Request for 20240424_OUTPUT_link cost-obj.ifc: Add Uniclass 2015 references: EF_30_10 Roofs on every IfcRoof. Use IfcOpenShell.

First a look at what the model holds.

```python
import ifcopenshell

model = ifcopenshell.open("20240424_OUTPUT_link cost-obj.ifc")
print(model.schema)
print("classifications:", [c.Name for c in model.by_type("IfcClassification")])
for ifc_class in ("IfcDoor", "IfcRoof", "IfcStair", "IfcWall", "IfcWindow"):
    print(ifc_class, len(model.by_type(ifc_class)))
```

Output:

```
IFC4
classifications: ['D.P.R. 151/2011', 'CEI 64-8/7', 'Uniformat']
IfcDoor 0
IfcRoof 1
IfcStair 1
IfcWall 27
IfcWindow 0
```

```python
import ifcopenshell
import ifcopenshell.api.classification

model = ifcopenshell.open("20240424_OUTPUT_link cost-obj.ifc")

system = ifcopenshell.api.classification.add_classification(model, classification="Uniclass 2015")

codes = {
    "IfcRoof": ("EF_30_10", "Roofs"),
}
for ifc_class, (code, name) in codes.items():
    products = model.by_type(ifc_class)
    ifcopenshell.api.classification.add_reference(
        model, products=products, classification=system, identification=code, name=name
    )
    print(code, len(products))

model.write("20240424_OUTPUT_link cost-obj_rev.ifc")
```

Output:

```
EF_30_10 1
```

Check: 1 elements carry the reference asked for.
